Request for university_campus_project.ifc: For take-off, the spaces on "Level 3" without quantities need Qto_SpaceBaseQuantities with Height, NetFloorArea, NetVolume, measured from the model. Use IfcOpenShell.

First a look at what the model holds.

```python
import ifcopenshell
import ifcopenshell.util.element
import ifcopenshell.util.unit

model = ifcopenshell.open("university_campus_project.ifc")
print(model.schema)
for unit_type in ("LENGTHUNIT", "AREAUNIT", "VOLUMEUNIT"):
    print(unit_type, ifcopenshell.util.unit.calculate_unit_scale(model, unit_type))
storey = next(s for s in model.by_type("IfcBuildingStorey") if s.Name == "Level 3")
spaces = [e for e in ifcopenshell.util.element.get_decomposition(storey) if e.is_a("IfcSpace")]
for e in sorted(spaces, key=lambda e: e.id()):
    print(e.id(), e.is_a(), e.Name, list(ifcopenshell.util.element.get_psets(e, qtos_only=True)), sep=" | ")
```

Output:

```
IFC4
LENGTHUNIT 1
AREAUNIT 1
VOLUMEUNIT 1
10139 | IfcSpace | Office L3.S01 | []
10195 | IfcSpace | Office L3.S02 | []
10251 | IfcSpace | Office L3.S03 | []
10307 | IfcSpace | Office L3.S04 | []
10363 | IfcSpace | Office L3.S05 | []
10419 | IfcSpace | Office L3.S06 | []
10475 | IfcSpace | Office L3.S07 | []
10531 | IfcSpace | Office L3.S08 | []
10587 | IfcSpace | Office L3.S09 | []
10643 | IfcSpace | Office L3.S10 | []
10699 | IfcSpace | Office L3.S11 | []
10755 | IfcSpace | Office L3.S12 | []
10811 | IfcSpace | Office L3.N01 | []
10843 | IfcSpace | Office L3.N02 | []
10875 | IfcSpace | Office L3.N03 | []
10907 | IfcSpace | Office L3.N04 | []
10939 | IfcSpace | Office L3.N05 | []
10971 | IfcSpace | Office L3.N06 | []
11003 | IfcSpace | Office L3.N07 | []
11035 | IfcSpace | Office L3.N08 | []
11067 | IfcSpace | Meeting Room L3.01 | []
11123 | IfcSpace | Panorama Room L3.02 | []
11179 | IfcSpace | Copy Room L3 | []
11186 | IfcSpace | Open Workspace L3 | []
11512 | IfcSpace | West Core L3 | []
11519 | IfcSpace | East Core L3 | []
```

```python
import ifcopenshell
import ifcopenshell.api.pset
import ifcopenshell.geom
import ifcopenshell.util.element
import ifcopenshell.util.shape
import ifcopenshell.util.unit

model = ifcopenshell.open("university_campus_project.ifc")
unit_scale = ifcopenshell.util.unit.calculate_unit_scale(model)
area_scale = ifcopenshell.util.unit.calculate_unit_scale(model, "AREAUNIT")
volume_scale = ifcopenshell.util.unit.calculate_unit_scale(model, "VOLUMEUNIT")
settings = ifcopenshell.geom.settings()

storey = next(s for s in model.by_type("IfcBuildingStorey") if s.Name == "Level 3")
spaces = [e for e in ifcopenshell.util.element.get_decomposition(storey) if e.is_a("IfcSpace")]

for e in sorted(spaces, key=lambda e: e.id()):
    if ifcopenshell.util.element.get_psets(e, qtos_only=True, should_inherit=False):
        continue
    # Geometry comes back in metres, in the element's own axes.
    shape = ifcopenshell.geom.create_shape(settings, e)
    values = {
        "Height": ifcopenshell.util.shape.get_z(shape.geometry) / unit_scale,
        "NetFloorArea": ifcopenshell.util.shape.get_footprint_area(shape.geometry) / area_scale,
        "NetVolume": ifcopenshell.util.shape.get_volume(shape.geometry) / volume_scale,
    }
    qto = ifcopenshell.api.pset.add_qto(model, product=e, name="Qto_SpaceBaseQuantities")
    ifcopenshell.api.pset.edit_qto(model, qto=qto, properties=values)
    print(e.id(), {k: round(v, 3) for k, v in values.items()})

model.write("university_campus_project_edited.ifc")
```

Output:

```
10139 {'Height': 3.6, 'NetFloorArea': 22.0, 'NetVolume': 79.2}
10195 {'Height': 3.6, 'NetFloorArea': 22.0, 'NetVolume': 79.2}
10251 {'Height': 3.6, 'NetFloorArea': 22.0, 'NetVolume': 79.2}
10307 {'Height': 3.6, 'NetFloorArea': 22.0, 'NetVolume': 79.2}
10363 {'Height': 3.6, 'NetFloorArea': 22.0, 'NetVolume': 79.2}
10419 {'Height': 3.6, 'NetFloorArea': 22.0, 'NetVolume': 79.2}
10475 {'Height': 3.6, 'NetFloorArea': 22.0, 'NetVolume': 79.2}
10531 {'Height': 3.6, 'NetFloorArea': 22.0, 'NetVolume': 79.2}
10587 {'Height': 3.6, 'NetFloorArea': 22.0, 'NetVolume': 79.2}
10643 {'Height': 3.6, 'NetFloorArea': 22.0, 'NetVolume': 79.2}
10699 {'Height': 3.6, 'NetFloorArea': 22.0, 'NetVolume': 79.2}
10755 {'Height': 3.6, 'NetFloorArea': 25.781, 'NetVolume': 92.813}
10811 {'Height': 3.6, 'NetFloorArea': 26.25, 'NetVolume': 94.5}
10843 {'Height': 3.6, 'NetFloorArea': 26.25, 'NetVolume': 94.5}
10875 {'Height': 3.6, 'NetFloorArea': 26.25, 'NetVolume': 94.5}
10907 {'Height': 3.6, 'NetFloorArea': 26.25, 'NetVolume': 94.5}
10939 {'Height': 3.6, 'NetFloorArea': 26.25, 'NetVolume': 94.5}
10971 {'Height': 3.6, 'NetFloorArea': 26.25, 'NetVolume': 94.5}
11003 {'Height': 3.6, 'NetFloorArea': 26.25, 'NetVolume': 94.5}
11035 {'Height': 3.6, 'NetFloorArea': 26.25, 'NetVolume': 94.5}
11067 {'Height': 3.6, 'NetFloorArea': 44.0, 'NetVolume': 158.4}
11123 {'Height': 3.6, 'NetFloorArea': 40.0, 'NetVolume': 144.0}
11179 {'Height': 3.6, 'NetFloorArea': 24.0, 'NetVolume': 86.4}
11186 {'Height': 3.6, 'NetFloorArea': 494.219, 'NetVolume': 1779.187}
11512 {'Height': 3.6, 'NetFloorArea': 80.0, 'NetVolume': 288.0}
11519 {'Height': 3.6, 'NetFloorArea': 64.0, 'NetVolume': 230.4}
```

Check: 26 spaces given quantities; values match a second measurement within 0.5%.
